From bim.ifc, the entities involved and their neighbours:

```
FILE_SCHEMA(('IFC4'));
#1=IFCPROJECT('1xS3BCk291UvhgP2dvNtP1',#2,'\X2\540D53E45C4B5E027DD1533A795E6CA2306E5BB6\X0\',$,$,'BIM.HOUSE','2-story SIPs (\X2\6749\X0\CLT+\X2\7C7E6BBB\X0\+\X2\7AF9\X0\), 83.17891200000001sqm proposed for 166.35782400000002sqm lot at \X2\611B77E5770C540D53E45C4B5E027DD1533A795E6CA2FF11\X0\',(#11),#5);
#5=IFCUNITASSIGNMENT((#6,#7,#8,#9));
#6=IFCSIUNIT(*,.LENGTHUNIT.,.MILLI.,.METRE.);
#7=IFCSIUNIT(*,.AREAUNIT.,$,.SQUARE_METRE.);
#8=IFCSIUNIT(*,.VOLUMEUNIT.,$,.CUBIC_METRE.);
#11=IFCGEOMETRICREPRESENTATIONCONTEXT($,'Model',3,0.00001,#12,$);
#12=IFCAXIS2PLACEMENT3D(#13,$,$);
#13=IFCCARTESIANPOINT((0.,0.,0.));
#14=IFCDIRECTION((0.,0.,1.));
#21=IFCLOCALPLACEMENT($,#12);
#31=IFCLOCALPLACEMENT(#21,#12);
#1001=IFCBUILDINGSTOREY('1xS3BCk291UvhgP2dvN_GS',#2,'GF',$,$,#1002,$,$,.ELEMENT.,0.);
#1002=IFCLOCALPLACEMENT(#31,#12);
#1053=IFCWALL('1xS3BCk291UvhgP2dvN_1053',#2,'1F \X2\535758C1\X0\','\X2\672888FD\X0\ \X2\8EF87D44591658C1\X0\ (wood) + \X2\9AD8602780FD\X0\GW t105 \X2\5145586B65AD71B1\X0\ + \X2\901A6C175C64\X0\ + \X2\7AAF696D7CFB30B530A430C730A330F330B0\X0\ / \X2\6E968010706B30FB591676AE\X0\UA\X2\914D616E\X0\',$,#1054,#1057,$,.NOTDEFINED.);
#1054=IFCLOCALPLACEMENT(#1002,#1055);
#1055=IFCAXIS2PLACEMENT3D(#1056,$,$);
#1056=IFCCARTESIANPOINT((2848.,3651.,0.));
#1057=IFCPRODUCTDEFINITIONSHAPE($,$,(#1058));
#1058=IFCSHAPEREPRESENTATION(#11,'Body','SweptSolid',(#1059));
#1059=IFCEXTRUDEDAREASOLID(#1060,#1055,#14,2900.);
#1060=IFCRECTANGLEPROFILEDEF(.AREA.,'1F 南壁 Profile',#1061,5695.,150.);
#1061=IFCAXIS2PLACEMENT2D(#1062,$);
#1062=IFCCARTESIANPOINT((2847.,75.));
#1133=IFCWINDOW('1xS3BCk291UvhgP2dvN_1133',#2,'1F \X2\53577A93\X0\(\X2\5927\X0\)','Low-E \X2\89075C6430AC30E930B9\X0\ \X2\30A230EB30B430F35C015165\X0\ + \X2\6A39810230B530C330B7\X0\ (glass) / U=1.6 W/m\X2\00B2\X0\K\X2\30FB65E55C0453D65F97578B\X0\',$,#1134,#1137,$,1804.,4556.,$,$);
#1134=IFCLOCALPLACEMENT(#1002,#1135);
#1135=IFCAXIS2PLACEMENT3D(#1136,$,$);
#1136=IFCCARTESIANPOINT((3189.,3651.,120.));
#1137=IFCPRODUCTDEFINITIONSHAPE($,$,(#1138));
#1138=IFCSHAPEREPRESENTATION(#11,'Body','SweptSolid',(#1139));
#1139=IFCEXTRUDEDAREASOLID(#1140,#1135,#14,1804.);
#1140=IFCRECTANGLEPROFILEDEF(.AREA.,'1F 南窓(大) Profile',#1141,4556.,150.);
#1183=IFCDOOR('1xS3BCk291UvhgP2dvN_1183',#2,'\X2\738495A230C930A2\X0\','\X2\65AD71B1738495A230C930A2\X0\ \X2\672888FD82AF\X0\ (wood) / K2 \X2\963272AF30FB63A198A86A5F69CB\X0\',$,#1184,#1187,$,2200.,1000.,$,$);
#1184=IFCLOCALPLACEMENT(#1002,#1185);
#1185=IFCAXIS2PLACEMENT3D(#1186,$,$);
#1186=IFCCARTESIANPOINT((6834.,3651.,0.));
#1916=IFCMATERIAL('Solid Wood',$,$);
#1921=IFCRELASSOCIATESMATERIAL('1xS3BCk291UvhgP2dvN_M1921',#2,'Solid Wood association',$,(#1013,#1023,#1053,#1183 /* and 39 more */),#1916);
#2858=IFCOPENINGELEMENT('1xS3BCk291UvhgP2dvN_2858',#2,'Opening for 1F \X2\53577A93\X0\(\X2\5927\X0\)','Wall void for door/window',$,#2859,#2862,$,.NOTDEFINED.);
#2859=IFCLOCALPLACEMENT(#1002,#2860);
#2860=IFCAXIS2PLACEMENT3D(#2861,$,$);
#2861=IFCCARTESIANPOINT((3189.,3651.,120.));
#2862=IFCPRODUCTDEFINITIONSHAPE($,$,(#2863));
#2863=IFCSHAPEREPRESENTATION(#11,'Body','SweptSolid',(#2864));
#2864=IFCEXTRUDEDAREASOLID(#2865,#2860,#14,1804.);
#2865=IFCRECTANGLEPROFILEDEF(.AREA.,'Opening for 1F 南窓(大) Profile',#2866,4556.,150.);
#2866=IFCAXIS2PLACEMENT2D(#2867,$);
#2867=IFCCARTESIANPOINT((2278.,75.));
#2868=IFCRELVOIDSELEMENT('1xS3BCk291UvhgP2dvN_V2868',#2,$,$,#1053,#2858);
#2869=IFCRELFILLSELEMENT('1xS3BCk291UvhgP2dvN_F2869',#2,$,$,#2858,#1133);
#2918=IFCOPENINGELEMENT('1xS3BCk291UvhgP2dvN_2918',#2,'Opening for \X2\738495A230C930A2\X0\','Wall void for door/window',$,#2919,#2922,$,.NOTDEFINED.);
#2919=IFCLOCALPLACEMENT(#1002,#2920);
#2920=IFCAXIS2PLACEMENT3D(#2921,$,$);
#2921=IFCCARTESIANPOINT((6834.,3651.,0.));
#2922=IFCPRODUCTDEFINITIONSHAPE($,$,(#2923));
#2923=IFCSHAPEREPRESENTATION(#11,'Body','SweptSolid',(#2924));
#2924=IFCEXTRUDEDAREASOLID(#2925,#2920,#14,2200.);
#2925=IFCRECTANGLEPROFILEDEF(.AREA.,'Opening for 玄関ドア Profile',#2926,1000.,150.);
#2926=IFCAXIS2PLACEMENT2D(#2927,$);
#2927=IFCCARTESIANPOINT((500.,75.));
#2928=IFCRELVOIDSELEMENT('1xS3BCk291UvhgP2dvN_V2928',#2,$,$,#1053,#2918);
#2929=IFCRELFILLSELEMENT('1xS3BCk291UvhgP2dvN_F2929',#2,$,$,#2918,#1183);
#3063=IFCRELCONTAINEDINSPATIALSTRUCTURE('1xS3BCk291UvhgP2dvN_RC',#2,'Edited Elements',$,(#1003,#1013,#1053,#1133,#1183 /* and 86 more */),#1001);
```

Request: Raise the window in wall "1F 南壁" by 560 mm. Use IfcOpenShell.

```python
import numpy as np
import ifcopenshell
import ifcopenshell.api.geometry
import ifcopenshell.util.placement
import ifcopenshell.util.unit

model = ifcopenshell.open("bim.ifc")
unit_scale = ifcopenshell.util.unit.calculate_unit_scale(model)

window = model.by_guid("1xS3BCk291UvhgP2dvN_1133")
opening = window.FillsVoids[0].RelatingOpeningElement
dz = 560.0

shift = np.array([0.0, 0.0, dz])
# The window is not placed relative to its opening, so move both.
for product in (opening, window):
    matrix = ifcopenshell.util.placement.get_local_placement(product.ObjectPlacement)
    matrix[:3, 3] += shift
    ifcopenshell.api.geometry.edit_object_placement(model, product=product, matrix=matrix, is_si=False)

print(f"moved by {dz * unit_scale:+.3f} m")

model.write("bim_edited.ifc")
```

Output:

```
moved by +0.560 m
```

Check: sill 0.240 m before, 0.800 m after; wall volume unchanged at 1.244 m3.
